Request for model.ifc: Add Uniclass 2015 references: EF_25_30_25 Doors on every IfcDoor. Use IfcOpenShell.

First a look at what the model holds.

```python
import ifcopenshell

model = ifcopenshell.open("model.ifc")
print(model.schema)
print("classifications:", [c.Name for c in model.by_type("IfcClassification")])
for ifc_class in ("IfcDoor", "IfcRoof", "IfcStair", "IfcWall", "IfcWindow"):
    print(ifc_class, len(model.by_type(ifc_class)))
```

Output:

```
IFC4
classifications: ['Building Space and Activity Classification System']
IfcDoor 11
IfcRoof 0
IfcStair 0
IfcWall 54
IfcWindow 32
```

```python
import ifcopenshell
import ifcopenshell.api.classification

model = ifcopenshell.open("model.ifc")

system = ifcopenshell.api.classification.add_classification(model, classification="Uniclass 2015")

codes = {
    "IfcDoor": ("EF_25_30_25", "Doors"),
}
for ifc_class, (code, name) in codes.items():
    products = model.by_type(ifc_class)
    ifcopenshell.api.classification.add_reference(
        model, products=products, classification=system, identification=code, name=name
    )
    print(code, len(products))

model.write("model_rev.ifc")
```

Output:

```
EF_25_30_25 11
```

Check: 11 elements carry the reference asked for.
